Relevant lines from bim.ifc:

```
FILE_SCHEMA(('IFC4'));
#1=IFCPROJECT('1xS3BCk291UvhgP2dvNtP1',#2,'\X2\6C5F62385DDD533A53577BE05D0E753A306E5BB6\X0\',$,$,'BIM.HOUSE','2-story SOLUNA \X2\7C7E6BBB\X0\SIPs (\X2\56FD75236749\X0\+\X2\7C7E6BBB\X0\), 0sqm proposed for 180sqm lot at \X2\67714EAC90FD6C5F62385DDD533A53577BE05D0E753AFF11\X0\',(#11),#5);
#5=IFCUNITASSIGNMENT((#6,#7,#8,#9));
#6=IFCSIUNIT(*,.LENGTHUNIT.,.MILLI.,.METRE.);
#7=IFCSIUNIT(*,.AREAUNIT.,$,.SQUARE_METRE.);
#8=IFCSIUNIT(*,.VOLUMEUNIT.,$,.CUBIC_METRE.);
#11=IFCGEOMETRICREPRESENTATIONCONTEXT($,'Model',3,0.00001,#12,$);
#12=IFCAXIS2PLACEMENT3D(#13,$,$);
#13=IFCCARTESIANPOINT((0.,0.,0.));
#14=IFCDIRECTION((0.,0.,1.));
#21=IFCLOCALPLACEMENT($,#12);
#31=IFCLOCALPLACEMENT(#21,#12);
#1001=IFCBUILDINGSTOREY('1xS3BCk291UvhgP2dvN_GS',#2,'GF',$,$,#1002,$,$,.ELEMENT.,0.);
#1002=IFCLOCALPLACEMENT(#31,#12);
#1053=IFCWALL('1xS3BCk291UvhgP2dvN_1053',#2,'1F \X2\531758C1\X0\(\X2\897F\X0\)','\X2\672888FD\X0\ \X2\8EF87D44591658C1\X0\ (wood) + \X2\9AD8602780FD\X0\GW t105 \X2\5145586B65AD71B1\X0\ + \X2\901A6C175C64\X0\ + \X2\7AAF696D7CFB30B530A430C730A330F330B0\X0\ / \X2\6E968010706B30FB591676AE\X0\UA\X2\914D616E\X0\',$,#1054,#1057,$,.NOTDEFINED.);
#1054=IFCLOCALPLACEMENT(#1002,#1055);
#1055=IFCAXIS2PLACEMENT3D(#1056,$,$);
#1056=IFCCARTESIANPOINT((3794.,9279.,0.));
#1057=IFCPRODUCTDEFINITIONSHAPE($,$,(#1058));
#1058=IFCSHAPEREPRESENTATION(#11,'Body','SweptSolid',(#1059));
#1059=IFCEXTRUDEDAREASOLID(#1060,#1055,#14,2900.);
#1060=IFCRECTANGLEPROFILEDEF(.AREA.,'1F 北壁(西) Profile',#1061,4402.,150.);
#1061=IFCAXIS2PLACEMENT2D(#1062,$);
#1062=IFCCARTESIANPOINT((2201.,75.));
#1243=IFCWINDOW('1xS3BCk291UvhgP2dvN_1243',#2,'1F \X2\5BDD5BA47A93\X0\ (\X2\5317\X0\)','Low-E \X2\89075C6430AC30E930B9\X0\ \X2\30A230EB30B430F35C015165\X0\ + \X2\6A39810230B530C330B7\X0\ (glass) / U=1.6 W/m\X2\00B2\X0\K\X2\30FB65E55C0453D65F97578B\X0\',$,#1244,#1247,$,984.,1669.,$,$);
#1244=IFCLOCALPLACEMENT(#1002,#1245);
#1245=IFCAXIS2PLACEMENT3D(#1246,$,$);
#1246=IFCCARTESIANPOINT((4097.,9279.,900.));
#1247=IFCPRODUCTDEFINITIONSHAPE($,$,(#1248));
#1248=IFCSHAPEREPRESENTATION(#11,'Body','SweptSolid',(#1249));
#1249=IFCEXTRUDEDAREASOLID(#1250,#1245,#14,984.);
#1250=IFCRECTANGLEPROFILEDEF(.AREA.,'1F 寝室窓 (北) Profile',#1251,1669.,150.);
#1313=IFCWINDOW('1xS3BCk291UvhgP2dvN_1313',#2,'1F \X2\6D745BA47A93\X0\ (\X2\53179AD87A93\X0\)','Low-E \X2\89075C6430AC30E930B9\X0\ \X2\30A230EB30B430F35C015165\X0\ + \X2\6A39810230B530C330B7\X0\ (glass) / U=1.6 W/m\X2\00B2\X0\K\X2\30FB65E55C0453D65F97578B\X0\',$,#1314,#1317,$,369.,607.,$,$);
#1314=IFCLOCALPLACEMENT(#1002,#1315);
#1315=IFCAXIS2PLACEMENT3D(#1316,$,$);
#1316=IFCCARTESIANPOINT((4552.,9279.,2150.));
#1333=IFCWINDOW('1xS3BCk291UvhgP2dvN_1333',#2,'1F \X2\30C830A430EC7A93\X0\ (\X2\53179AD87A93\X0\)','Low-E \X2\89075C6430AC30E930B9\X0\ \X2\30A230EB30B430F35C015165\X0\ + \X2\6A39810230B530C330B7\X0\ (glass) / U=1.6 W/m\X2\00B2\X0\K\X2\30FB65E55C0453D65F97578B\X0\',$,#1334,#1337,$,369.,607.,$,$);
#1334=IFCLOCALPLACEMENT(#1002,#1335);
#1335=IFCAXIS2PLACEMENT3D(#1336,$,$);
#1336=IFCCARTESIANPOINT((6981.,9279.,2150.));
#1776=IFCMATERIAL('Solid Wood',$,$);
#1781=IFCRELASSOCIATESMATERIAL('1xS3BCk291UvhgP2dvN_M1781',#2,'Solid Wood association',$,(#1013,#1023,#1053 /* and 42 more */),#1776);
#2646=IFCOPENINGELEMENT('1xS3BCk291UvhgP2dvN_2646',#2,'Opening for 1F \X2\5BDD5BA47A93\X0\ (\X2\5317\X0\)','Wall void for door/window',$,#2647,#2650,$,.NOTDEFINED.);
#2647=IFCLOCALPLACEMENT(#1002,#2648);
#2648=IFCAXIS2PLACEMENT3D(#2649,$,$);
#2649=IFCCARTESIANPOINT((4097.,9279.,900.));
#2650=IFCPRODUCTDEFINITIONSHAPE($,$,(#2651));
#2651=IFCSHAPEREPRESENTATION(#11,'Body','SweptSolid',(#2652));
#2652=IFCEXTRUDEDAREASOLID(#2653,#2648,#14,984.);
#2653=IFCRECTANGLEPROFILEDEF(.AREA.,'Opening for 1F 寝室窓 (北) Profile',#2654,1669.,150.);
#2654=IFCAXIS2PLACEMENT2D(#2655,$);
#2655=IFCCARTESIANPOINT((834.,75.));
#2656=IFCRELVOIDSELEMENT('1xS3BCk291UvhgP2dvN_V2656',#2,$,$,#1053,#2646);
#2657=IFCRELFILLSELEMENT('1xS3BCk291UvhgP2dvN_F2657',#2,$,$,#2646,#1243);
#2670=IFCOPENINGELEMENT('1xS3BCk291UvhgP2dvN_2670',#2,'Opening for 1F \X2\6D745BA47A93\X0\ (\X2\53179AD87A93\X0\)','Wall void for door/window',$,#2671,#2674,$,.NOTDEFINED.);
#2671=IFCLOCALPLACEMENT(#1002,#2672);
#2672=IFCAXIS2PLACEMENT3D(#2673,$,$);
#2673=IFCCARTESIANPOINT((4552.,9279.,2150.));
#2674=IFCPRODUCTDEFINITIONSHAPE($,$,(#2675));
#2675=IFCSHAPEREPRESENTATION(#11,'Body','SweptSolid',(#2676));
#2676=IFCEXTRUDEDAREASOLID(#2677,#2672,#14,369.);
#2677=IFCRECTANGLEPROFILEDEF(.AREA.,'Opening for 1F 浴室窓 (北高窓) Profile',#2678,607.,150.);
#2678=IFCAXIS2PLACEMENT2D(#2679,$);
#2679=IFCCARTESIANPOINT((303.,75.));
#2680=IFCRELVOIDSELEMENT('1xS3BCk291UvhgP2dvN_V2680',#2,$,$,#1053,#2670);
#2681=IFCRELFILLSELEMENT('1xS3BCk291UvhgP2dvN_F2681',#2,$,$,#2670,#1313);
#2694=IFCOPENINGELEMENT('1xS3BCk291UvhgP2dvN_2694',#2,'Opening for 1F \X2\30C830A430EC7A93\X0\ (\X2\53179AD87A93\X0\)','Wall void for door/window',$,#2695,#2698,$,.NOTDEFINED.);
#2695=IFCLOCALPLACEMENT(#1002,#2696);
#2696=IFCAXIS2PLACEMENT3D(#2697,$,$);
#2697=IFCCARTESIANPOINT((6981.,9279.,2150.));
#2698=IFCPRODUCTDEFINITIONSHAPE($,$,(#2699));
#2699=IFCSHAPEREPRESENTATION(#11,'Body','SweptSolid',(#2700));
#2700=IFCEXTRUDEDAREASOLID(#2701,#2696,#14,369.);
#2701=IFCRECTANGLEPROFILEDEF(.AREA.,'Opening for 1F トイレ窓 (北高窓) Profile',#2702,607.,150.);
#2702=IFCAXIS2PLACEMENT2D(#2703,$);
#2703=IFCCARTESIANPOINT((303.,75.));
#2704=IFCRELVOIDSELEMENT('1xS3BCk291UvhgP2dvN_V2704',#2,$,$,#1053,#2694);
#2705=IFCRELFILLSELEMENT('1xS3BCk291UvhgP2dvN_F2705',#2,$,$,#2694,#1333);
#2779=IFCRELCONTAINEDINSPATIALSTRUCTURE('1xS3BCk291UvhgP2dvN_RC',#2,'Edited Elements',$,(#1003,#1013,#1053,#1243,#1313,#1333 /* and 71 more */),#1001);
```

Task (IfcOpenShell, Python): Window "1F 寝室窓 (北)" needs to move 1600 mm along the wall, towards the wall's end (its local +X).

```python
import ifcopenshell
import ifcopenshell.api.geometry
import ifcopenshell.util.placement
import ifcopenshell.util.unit

model = ifcopenshell.open("bim.ifc")
unit_scale = ifcopenshell.util.unit.calculate_unit_scale(model)

window = model.by_guid("1xS3BCk291UvhgP2dvN_1243")
opening = window.FillsVoids[0].RelatingOpeningElement
wall = opening.VoidsElements[0].RelatingBuildingElement

wall_matrix = ifcopenshell.util.placement.get_local_placement(wall.ObjectPlacement)
shift = wall_matrix[:3, 0] * 1.6 / unit_scale
before = ifcopenshell.util.placement.get_local_placement(window.ObjectPlacement)[:3, 3].copy()

# The window is not placed relative to its opening, so move both.
for product in (opening, window):
    matrix = ifcopenshell.util.placement.get_local_placement(product.ObjectPlacement)
    matrix[:3, 3] += shift
    ifcopenshell.api.geometry.edit_object_placement(model, product=product, matrix=matrix, is_si=False)

after = ifcopenshell.util.placement.get_local_placement(window.ObjectPlacement)[:3, 3]
print("window moved by", (after - before).round(3) + 0.0)

model.write("bim_edited.ifc")
```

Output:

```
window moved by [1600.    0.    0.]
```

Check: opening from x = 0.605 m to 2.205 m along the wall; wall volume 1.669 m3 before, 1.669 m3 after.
